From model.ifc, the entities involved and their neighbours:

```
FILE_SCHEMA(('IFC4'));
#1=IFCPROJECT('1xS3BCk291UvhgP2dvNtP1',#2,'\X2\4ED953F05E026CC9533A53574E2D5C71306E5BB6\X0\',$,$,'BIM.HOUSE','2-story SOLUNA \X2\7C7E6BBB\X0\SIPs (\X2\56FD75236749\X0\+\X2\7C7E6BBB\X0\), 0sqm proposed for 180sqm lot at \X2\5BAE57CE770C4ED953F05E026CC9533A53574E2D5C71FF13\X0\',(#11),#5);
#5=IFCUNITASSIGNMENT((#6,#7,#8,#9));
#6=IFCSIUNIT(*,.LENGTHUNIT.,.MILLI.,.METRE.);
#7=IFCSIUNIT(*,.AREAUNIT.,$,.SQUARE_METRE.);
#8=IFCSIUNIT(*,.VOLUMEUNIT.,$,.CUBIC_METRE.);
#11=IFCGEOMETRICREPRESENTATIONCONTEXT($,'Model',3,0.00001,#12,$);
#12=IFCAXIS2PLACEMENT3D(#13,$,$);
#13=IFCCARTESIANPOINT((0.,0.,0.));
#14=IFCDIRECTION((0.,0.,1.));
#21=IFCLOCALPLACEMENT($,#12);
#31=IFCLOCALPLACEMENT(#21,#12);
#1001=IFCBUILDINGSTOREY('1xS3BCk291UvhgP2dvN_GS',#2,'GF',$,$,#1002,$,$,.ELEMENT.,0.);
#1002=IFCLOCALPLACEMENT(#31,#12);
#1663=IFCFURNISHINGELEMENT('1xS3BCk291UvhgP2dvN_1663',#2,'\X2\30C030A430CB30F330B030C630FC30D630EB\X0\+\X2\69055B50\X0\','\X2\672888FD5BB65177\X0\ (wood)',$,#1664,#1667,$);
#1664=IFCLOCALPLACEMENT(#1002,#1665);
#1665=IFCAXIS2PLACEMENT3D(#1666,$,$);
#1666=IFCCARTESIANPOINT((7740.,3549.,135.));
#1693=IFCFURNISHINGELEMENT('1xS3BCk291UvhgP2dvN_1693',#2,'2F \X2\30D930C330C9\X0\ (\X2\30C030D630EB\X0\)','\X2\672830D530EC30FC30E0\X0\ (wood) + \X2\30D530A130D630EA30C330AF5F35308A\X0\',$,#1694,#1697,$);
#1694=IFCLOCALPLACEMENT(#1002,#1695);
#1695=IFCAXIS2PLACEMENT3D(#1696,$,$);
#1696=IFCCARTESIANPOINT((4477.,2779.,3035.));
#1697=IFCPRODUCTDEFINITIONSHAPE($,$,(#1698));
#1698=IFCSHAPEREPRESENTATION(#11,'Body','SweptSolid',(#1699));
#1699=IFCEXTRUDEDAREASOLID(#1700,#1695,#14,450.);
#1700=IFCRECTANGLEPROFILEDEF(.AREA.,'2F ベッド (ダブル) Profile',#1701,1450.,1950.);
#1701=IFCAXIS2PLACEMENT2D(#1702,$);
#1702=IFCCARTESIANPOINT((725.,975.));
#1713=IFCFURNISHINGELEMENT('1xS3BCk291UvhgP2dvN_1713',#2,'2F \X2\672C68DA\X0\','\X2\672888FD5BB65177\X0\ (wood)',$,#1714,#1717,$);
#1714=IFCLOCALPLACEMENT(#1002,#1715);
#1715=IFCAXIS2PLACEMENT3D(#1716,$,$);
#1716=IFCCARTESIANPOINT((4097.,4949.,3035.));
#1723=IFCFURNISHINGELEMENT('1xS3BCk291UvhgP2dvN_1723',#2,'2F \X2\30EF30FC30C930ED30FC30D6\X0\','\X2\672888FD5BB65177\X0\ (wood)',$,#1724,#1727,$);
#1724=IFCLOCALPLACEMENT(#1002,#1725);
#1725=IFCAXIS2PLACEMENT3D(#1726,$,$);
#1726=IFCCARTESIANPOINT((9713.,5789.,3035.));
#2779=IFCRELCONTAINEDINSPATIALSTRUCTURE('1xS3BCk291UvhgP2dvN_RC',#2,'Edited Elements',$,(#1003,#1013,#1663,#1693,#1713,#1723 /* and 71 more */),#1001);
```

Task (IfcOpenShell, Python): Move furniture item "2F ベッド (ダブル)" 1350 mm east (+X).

```python
import ifcopenshell
import ifcopenshell.api.geometry
import ifcopenshell.util.placement
import ifcopenshell.util.unit

model = ifcopenshell.open("model.ifc")
unit_scale = ifcopenshell.util.unit.calculate_unit_scale(model)

item = model.by_guid("1xS3BCk291UvhgP2dvN_1693")
matrix = ifcopenshell.util.placement.get_local_placement(item.ObjectPlacement)
matrix[0, 3] += 1.35 / unit_scale
ifcopenshell.api.geometry.edit_object_placement(model, product=item, matrix=matrix, is_si=False)

print(ifcopenshell.util.placement.get_local_placement(item.ObjectPlacement).round(3) + 0.0)

model.write("model_updated.ifc")
```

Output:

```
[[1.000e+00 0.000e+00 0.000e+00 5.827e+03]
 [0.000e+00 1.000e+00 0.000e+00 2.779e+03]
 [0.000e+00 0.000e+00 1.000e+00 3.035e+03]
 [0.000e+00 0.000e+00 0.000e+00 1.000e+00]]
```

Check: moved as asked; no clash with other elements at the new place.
